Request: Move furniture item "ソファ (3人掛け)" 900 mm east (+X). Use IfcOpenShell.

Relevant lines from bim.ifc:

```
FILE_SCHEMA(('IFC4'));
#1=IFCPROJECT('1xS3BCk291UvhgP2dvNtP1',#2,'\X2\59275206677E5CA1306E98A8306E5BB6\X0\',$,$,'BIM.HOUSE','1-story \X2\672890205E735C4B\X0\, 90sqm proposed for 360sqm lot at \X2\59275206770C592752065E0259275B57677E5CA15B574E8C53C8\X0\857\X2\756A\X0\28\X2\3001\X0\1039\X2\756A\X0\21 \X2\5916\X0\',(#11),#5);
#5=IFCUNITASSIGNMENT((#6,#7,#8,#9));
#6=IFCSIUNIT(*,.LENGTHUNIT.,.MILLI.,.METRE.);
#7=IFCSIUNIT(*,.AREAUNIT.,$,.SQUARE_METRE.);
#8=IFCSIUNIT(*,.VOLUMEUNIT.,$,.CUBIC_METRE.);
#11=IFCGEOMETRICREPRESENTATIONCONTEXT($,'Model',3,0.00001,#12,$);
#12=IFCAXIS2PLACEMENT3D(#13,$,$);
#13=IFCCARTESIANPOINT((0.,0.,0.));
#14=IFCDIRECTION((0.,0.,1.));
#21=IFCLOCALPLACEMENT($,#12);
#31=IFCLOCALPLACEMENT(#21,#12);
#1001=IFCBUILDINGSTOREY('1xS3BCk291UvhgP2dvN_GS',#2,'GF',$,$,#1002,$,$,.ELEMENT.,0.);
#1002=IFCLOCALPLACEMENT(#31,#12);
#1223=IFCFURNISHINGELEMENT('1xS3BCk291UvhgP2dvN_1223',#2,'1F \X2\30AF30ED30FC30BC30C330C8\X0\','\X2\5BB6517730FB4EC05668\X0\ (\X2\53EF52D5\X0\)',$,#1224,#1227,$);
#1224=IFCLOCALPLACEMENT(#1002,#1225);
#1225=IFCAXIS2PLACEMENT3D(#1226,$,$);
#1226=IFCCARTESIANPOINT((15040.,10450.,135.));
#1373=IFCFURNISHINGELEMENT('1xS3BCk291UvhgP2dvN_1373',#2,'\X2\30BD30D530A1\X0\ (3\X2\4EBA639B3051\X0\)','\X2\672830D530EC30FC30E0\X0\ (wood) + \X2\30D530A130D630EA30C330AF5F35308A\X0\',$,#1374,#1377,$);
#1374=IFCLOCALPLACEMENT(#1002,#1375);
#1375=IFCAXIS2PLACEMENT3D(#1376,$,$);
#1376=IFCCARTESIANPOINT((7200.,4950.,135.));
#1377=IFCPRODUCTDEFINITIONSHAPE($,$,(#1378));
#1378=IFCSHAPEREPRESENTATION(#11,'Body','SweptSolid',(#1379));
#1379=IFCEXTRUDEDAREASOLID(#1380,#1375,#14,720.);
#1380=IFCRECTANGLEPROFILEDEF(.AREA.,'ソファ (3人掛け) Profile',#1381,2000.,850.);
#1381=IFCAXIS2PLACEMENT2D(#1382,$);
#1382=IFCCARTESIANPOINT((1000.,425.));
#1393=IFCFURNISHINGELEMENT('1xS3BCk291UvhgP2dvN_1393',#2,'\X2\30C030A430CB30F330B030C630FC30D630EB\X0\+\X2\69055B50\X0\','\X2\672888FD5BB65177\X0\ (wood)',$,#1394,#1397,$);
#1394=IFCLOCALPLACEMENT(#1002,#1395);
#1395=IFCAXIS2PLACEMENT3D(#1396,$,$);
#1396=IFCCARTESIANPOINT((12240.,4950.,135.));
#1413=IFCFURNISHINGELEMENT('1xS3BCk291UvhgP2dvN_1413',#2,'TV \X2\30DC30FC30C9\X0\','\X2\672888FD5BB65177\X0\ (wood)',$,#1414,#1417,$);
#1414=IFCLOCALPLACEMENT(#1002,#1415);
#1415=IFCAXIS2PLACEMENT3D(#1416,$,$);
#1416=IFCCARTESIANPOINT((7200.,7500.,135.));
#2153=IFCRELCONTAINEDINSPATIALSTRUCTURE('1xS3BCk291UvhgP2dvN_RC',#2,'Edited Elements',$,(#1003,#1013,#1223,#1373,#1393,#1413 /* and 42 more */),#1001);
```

```python
import ifcopenshell
import ifcopenshell.api.geometry
import ifcopenshell.util.placement

model = ifcopenshell.open("bim.ifc")

item = model.by_guid("1xS3BCk291UvhgP2dvN_1373")
matrix = ifcopenshell.util.placement.get_local_placement(item.ObjectPlacement)
matrix[0, 3] += 900.0
ifcopenshell.api.geometry.edit_object_placement(model, product=item, matrix=matrix, is_si=False)

print(ifcopenshell.util.placement.get_local_placement(item.ObjectPlacement).round(3) + 0.0)

model.write("bim_updated.ifc")
```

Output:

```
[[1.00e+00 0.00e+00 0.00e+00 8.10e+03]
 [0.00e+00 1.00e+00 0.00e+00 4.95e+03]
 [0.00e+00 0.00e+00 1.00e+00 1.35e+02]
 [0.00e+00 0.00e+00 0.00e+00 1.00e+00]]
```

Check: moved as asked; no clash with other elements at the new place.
